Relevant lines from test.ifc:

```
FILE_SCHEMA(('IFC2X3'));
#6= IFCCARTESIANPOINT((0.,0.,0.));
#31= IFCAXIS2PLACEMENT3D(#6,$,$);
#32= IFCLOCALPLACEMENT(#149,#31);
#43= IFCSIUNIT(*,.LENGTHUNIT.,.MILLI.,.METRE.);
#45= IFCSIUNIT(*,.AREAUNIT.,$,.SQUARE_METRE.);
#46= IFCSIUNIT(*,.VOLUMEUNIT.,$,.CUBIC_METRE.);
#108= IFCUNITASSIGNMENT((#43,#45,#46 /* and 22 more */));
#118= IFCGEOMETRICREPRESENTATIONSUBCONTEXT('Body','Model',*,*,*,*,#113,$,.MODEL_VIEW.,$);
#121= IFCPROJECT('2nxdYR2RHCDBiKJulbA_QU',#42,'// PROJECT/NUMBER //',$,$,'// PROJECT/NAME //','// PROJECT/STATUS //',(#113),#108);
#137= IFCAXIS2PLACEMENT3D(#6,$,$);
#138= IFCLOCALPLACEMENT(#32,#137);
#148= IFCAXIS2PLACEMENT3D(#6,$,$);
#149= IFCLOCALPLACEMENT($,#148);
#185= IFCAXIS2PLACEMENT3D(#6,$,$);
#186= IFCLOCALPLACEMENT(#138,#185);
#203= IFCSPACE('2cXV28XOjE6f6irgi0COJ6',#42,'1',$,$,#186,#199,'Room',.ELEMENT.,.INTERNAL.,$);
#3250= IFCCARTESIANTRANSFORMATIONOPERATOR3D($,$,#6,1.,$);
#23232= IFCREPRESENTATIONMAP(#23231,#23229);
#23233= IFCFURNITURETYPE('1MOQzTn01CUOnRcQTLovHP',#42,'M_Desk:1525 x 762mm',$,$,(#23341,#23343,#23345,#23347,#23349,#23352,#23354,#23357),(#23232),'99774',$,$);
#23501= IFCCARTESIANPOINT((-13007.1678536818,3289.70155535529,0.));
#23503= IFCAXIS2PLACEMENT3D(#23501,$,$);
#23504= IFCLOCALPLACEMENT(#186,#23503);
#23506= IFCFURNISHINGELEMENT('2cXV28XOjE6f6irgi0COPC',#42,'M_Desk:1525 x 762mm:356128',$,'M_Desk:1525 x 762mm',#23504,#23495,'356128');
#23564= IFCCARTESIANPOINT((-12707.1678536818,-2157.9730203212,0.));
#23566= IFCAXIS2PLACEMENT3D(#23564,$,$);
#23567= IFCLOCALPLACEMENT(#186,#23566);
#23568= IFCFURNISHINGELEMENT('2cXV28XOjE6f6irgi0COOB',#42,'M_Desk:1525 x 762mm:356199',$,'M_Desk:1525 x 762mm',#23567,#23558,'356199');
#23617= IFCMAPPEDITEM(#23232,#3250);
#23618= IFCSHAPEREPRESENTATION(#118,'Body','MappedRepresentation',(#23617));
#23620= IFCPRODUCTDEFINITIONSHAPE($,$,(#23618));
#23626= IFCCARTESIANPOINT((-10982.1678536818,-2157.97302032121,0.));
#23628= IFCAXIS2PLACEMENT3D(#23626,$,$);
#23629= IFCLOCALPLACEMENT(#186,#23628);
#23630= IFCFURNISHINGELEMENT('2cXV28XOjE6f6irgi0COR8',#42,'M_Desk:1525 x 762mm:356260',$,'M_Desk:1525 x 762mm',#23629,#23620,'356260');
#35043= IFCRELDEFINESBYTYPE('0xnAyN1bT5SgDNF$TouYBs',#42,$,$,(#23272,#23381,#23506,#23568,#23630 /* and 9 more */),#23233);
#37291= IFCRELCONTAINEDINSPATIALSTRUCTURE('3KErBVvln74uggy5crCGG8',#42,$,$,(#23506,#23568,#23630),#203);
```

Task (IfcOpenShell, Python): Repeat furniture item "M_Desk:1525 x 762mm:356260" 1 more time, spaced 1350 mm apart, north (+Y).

```python
import numpy as np
import ifcopenshell
import ifcopenshell.api.geometry
import ifcopenshell.api.root
import ifcopenshell.util.element
import ifcopenshell.util.placement
import ifcopenshell.util.unit

model = ifcopenshell.open("test.ifc")
unit_scale = ifcopenshell.util.unit.calculate_unit_scale(model)


def reuse_history(source, copy):
    """copy_class also copies each property set's owner history, people and application; keep the originals."""
    for rel in copy.IsDefinedBy:
        if rel.is_a("IfcRelDefinesByProperties") and (history := rel.RelatingPropertyDefinition.OwnerHistory):
            rel.RelatingPropertyDefinition.OwnerHistory = source.OwnerHistory
            ifcopenshell.util.element.remove_deep2(model, history)


source = model.by_guid("2cXV28XOjE6f6irgi0COR8")
base = ifcopenshell.util.placement.get_local_placement(source.ObjectPlacement)
step = np.array([0.0, 1.0, 0.0]) * 1.35 / unit_scale

for i in range(1, 2):
    copy = ifcopenshell.api.root.copy_class(model, product=source)
    copy.Representation = ifcopenshell.util.element.copy_deep(
        model, source.Representation, exclude=["IfcGeometricRepresentationContext", "IfcRepresentationMap"]
    )
    copy.Name = "M_Desk:1525 x 762mm"
    copy.Tag = None
    reuse_history(source, copy)
    matrix = base.copy()
    matrix[:3, 3] += i * step
    print("added at", matrix[:3, 3].round(3) + 0.0)
    ifcopenshell.api.geometry.edit_object_placement(model, product=copy, matrix=matrix, is_si=False)

model.write("test_rev.ifc")
```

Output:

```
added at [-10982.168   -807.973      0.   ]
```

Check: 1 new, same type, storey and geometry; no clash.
